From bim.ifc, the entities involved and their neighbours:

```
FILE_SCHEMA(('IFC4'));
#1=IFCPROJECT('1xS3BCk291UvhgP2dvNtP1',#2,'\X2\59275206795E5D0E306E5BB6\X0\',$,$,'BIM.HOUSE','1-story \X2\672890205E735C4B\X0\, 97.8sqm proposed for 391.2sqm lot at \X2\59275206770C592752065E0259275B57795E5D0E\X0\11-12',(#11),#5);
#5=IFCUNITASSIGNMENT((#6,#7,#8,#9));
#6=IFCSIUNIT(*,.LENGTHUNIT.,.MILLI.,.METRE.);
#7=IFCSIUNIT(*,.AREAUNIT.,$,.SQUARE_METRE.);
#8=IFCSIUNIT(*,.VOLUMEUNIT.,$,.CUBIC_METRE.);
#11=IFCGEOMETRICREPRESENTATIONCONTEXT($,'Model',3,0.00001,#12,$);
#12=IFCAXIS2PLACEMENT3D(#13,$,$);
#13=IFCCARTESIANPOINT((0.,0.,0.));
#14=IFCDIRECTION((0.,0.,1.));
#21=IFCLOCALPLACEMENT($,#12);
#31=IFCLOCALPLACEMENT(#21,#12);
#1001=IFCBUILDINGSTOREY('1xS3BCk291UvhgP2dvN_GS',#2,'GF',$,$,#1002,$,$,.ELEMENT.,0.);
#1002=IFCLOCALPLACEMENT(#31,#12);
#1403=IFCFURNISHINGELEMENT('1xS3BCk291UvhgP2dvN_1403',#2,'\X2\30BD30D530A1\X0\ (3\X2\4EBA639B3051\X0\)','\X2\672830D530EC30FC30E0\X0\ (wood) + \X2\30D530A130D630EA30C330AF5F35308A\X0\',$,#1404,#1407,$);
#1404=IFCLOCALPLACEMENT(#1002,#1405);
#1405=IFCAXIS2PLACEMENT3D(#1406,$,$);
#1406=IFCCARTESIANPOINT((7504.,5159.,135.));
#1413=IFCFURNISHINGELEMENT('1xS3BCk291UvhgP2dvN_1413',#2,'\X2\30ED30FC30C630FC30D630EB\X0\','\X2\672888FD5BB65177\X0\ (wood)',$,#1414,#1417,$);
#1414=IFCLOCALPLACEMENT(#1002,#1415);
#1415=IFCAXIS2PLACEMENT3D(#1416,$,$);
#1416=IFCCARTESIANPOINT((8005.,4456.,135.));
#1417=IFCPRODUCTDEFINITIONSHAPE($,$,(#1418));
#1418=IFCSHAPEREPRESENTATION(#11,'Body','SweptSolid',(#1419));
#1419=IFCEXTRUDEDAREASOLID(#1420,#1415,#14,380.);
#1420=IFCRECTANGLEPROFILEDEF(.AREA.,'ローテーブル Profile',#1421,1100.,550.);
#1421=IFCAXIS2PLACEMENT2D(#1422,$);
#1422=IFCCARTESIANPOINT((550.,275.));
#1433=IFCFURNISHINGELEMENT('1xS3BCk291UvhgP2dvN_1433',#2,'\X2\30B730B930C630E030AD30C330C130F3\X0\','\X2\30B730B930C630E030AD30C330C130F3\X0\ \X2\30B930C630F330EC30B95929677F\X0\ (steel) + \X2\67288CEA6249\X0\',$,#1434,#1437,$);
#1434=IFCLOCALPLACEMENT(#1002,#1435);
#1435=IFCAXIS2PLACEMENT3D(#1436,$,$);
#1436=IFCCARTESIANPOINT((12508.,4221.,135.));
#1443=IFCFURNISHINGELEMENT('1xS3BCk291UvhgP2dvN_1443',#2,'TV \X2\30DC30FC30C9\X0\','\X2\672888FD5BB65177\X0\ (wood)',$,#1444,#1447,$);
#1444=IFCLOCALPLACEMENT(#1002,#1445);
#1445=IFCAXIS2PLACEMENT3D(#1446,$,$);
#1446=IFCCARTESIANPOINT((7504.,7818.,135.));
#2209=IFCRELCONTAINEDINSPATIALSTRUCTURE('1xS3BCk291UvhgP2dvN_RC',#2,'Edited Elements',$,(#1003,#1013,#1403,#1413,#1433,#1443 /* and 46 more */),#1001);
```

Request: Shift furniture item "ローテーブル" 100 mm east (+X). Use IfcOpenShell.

```python
import ifcopenshell
import ifcopenshell.api.geometry
import ifcopenshell.util.placement

model = ifcopenshell.open("bim.ifc")

item = model.by_guid("1xS3BCk291UvhgP2dvN_1413")
matrix = ifcopenshell.util.placement.get_local_placement(item.ObjectPlacement)
matrix[0, 3] += 100.0
ifcopenshell.api.geometry.edit_object_placement(model, product=item, matrix=matrix, is_si=False)

print(ifcopenshell.util.placement.get_local_placement(item.ObjectPlacement).round(3) + 0.0)

model.write("bim_updated.ifc")
```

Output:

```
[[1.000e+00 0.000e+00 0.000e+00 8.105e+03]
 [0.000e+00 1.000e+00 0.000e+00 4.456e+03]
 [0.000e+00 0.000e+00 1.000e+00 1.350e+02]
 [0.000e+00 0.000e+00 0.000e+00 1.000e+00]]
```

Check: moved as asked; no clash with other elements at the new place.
